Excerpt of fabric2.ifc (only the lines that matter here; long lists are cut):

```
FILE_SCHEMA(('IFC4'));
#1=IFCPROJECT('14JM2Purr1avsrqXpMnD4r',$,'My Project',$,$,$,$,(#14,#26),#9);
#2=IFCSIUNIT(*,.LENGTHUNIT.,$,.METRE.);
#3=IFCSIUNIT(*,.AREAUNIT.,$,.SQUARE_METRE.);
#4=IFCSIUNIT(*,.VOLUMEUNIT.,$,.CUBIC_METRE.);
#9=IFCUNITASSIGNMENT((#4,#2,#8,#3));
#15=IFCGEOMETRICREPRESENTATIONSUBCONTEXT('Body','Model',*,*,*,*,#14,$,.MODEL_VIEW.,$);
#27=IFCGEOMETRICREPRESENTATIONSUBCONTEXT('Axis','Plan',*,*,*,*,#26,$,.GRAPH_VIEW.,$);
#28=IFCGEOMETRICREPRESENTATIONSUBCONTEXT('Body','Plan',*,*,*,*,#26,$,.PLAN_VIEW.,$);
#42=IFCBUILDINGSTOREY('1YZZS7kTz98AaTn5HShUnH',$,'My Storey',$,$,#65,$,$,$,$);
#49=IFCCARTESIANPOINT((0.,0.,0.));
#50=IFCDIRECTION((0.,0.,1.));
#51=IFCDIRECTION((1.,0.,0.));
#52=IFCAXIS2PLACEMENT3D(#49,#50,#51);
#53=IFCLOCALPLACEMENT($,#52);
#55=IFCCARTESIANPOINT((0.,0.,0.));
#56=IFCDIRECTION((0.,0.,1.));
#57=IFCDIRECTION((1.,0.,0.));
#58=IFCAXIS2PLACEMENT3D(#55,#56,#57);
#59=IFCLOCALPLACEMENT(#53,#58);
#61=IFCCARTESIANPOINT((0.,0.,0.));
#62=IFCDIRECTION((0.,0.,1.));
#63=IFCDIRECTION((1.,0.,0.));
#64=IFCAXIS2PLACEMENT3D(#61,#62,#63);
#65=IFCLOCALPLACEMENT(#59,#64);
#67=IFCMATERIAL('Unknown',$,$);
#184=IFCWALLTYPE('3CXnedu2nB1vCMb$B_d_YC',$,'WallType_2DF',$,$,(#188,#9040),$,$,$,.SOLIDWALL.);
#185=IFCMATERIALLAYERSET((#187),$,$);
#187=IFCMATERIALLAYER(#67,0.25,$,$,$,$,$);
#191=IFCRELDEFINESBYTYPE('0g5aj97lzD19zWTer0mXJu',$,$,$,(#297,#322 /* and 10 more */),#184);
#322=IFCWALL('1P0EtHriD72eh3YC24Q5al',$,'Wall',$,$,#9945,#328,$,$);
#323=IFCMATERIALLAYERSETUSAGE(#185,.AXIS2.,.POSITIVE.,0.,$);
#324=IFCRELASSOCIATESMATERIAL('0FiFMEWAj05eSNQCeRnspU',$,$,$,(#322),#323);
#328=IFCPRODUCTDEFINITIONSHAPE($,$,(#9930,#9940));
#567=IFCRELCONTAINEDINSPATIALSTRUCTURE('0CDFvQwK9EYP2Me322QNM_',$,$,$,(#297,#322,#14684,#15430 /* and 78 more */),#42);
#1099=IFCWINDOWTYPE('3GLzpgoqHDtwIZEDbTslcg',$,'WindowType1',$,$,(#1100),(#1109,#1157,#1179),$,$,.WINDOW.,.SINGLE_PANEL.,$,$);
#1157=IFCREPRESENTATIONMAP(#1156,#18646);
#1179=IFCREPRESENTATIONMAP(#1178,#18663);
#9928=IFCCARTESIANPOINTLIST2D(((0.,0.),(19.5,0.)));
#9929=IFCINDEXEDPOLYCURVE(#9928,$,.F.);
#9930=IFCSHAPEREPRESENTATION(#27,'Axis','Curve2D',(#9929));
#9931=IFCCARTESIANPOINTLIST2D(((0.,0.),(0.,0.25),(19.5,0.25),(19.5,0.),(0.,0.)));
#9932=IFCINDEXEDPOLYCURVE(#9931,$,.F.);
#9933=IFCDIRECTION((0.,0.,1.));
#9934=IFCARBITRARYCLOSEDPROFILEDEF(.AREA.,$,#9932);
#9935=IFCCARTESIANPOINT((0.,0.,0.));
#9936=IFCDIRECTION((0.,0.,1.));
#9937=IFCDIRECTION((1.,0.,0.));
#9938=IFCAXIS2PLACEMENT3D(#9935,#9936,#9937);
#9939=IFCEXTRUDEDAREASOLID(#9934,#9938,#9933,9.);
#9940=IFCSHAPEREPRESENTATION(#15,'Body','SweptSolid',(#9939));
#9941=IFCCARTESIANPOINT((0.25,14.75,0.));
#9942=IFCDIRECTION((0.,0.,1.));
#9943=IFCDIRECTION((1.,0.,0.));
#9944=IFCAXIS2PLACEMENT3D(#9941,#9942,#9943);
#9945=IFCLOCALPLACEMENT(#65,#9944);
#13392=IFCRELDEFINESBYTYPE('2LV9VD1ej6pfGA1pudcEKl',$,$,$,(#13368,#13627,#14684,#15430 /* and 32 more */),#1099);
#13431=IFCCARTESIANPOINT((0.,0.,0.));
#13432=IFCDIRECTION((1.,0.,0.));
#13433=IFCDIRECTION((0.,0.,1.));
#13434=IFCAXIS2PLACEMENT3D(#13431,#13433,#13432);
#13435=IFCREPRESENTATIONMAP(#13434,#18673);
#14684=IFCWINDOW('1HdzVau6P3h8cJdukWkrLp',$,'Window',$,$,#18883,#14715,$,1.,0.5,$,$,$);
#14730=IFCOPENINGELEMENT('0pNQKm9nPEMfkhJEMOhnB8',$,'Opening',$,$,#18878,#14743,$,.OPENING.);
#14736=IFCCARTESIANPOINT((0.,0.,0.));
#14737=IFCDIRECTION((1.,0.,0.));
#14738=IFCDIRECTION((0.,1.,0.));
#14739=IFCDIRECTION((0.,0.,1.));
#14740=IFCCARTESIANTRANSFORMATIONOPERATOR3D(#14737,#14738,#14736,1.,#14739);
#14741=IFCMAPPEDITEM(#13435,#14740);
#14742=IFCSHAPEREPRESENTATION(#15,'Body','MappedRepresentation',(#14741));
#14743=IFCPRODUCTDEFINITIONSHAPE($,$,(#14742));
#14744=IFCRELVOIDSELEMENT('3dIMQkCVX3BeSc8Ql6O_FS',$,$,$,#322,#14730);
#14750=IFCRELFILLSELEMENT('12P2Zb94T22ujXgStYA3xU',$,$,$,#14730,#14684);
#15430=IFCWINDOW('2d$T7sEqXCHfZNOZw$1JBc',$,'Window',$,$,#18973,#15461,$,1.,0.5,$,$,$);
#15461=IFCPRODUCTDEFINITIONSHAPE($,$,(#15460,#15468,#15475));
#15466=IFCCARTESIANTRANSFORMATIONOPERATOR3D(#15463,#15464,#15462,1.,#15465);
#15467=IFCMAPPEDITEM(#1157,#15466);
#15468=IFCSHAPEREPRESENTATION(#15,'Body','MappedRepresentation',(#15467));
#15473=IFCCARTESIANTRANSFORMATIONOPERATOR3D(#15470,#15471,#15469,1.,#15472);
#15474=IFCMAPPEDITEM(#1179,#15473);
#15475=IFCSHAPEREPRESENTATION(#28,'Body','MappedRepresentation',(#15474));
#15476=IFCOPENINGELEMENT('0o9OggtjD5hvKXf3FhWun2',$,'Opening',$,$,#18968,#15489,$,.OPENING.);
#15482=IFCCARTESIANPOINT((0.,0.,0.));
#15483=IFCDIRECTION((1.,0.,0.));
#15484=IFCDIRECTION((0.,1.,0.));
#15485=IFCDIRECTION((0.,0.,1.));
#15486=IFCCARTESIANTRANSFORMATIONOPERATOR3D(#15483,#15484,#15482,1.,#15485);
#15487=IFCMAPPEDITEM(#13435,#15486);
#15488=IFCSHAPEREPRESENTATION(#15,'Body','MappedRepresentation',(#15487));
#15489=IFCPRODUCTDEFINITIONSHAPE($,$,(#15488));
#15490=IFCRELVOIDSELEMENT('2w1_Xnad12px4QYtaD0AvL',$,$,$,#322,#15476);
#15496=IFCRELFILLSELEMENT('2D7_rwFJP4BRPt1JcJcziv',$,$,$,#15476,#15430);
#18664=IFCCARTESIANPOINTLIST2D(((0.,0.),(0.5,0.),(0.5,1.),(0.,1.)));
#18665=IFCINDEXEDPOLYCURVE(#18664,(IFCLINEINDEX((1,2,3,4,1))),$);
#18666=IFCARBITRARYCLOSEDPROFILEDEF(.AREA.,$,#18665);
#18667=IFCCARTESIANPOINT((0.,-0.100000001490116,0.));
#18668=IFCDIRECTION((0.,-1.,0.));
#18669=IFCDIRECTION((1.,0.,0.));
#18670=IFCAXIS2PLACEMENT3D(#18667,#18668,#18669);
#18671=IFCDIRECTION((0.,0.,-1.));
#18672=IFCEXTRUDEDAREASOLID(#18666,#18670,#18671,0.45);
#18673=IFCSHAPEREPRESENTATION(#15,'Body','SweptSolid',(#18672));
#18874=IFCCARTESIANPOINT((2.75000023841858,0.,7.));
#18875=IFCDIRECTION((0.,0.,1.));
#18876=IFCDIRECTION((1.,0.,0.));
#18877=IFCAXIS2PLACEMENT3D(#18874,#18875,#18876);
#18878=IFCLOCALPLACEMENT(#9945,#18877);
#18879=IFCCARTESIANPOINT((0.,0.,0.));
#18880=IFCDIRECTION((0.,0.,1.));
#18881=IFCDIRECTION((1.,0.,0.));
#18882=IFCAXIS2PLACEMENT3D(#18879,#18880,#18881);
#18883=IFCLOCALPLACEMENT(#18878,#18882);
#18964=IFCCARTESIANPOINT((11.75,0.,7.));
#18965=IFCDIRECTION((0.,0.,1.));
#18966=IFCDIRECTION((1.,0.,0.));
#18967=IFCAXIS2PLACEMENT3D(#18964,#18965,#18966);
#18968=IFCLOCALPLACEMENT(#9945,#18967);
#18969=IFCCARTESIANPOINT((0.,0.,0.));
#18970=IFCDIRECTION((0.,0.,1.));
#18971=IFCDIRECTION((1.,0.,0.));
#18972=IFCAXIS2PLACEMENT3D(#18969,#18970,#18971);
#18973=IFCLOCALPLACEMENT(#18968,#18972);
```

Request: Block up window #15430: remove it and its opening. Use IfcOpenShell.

```python
import ifcopenshell
import ifcopenshell.api.feature
import ifcopenshell.api.root
import ifcopenshell.geom
import ifcopenshell.util.shape

model = ifcopenshell.open("fabric2.ifc")
settings = ifcopenshell.geom.settings()


def volume(element):
    """Net volume in cubic metres, openings subtracted."""
    shape = ifcopenshell.geom.create_shape(settings, element)
    return ifcopenshell.util.shape.get_volume(shape.geometry)


window = model.by_guid("2d$T7sEqXCHfZNOZw$1JBc")
opening = window.FillsVoids[0].RelatingOpeningElement
wall = opening.VoidsElements[0].RelatingBuildingElement
before = volume(wall)

ifcopenshell.api.root.remove_product(model, product=window)
ifcopenshell.api.feature.remove_feature(model, feature=opening)

after = volume(wall)

print(f"wall volume {before:.3f} -> {after:.3f} m3")

model.write("fabric2_edited.ifc")
```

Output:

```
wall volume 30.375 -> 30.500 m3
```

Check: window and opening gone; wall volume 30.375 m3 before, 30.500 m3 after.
